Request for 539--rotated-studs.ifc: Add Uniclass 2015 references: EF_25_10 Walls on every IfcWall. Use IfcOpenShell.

First a look at what the model holds.

```python
import ifcopenshell

model = ifcopenshell.open("539--rotated-studs.ifc")
print(model.schema)
print("classifications:", [c.Name for c in model.by_type("IfcClassification")])
for ifc_class in ("IfcDoor", "IfcRoof", "IfcStair", "IfcWall", "IfcWindow"):
    print(ifc_class, len(model.by_type(ifc_class)))
```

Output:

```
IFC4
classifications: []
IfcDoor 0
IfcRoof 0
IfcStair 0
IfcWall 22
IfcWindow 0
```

```python
import ifcopenshell
import ifcopenshell.api.classification

model = ifcopenshell.open("539--rotated-studs.ifc")

system = ifcopenshell.api.classification.add_classification(model, classification="Uniclass 2015")

codes = {
    "IfcWall": ("EF_25_10", "Walls"),
}
for ifc_class, (code, name) in codes.items():
    products = model.by_type(ifc_class)
    ifcopenshell.api.classification.add_reference(
        model, products=products, classification=system, identification=code, name=name
    )
    print(code, len(products))

model.write("539--rotated-studs-out.ifc")
```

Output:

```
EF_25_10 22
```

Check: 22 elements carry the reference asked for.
